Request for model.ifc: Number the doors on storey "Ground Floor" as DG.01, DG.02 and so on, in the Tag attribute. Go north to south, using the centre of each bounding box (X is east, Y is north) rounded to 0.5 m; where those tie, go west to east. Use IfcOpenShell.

First a look at what the model holds.

```python
import ifcopenshell
import ifcopenshell.util.element
import ifcopenshell.util.placement

model = ifcopenshell.open("model.ifc")
print(model.schema)
storey = next(s for s in model.by_type("IfcBuildingStorey") if s.Name == "Ground Floor")
doors = [e for e in ifcopenshell.util.element.get_decomposition(storey) if e.is_a("IfcDoor")]
for e in sorted(doors, key=lambda e: e.id()):
    origin = ifcopenshell.util.placement.get_local_placement(e.ObjectPlacement)[:3, 3]
    print(e.id(), e.Tag, e.Name, origin.round(2) + 0.0, sep=" | ")
```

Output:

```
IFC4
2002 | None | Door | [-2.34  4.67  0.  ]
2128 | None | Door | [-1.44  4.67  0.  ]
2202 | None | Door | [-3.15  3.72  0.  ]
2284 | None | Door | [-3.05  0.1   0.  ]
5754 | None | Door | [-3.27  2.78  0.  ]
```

```python
import ifcopenshell
import ifcopenshell.geom
import ifcopenshell.util.element
import ifcopenshell.util.shape

model = ifcopenshell.open("model.ifc")
settings = ifcopenshell.geom.settings()
settings.set("use-world-coords", True)


def centre(element):
    shape = ifcopenshell.geom.create_shape(settings, element)
    return ifcopenshell.util.shape.get_bbox_centroid(shape.geometry)


storey = next(s for s in model.by_type("IfcBuildingStorey") if s.Name == "Ground Floor")
doors = [e for e in ifcopenshell.util.element.get_decomposition(storey) if e.is_a("IfcDoor")]

# Insertion points can sit at a corner or the storey origin, so sort by the geometry (in metres).
centres = {e: centre(e) for e in doors}
doors.sort(key=lambda e: (-round(centres[e][1] / 0.5), centres[e][0]))

for i, e in enumerate(doors, start=1):
    number = f"DG.{i:02d}"
    e.Tag = number
    print(e.id(), number)

model.write("model-out.ifc")
```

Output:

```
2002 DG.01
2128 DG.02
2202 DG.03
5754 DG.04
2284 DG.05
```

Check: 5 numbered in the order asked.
